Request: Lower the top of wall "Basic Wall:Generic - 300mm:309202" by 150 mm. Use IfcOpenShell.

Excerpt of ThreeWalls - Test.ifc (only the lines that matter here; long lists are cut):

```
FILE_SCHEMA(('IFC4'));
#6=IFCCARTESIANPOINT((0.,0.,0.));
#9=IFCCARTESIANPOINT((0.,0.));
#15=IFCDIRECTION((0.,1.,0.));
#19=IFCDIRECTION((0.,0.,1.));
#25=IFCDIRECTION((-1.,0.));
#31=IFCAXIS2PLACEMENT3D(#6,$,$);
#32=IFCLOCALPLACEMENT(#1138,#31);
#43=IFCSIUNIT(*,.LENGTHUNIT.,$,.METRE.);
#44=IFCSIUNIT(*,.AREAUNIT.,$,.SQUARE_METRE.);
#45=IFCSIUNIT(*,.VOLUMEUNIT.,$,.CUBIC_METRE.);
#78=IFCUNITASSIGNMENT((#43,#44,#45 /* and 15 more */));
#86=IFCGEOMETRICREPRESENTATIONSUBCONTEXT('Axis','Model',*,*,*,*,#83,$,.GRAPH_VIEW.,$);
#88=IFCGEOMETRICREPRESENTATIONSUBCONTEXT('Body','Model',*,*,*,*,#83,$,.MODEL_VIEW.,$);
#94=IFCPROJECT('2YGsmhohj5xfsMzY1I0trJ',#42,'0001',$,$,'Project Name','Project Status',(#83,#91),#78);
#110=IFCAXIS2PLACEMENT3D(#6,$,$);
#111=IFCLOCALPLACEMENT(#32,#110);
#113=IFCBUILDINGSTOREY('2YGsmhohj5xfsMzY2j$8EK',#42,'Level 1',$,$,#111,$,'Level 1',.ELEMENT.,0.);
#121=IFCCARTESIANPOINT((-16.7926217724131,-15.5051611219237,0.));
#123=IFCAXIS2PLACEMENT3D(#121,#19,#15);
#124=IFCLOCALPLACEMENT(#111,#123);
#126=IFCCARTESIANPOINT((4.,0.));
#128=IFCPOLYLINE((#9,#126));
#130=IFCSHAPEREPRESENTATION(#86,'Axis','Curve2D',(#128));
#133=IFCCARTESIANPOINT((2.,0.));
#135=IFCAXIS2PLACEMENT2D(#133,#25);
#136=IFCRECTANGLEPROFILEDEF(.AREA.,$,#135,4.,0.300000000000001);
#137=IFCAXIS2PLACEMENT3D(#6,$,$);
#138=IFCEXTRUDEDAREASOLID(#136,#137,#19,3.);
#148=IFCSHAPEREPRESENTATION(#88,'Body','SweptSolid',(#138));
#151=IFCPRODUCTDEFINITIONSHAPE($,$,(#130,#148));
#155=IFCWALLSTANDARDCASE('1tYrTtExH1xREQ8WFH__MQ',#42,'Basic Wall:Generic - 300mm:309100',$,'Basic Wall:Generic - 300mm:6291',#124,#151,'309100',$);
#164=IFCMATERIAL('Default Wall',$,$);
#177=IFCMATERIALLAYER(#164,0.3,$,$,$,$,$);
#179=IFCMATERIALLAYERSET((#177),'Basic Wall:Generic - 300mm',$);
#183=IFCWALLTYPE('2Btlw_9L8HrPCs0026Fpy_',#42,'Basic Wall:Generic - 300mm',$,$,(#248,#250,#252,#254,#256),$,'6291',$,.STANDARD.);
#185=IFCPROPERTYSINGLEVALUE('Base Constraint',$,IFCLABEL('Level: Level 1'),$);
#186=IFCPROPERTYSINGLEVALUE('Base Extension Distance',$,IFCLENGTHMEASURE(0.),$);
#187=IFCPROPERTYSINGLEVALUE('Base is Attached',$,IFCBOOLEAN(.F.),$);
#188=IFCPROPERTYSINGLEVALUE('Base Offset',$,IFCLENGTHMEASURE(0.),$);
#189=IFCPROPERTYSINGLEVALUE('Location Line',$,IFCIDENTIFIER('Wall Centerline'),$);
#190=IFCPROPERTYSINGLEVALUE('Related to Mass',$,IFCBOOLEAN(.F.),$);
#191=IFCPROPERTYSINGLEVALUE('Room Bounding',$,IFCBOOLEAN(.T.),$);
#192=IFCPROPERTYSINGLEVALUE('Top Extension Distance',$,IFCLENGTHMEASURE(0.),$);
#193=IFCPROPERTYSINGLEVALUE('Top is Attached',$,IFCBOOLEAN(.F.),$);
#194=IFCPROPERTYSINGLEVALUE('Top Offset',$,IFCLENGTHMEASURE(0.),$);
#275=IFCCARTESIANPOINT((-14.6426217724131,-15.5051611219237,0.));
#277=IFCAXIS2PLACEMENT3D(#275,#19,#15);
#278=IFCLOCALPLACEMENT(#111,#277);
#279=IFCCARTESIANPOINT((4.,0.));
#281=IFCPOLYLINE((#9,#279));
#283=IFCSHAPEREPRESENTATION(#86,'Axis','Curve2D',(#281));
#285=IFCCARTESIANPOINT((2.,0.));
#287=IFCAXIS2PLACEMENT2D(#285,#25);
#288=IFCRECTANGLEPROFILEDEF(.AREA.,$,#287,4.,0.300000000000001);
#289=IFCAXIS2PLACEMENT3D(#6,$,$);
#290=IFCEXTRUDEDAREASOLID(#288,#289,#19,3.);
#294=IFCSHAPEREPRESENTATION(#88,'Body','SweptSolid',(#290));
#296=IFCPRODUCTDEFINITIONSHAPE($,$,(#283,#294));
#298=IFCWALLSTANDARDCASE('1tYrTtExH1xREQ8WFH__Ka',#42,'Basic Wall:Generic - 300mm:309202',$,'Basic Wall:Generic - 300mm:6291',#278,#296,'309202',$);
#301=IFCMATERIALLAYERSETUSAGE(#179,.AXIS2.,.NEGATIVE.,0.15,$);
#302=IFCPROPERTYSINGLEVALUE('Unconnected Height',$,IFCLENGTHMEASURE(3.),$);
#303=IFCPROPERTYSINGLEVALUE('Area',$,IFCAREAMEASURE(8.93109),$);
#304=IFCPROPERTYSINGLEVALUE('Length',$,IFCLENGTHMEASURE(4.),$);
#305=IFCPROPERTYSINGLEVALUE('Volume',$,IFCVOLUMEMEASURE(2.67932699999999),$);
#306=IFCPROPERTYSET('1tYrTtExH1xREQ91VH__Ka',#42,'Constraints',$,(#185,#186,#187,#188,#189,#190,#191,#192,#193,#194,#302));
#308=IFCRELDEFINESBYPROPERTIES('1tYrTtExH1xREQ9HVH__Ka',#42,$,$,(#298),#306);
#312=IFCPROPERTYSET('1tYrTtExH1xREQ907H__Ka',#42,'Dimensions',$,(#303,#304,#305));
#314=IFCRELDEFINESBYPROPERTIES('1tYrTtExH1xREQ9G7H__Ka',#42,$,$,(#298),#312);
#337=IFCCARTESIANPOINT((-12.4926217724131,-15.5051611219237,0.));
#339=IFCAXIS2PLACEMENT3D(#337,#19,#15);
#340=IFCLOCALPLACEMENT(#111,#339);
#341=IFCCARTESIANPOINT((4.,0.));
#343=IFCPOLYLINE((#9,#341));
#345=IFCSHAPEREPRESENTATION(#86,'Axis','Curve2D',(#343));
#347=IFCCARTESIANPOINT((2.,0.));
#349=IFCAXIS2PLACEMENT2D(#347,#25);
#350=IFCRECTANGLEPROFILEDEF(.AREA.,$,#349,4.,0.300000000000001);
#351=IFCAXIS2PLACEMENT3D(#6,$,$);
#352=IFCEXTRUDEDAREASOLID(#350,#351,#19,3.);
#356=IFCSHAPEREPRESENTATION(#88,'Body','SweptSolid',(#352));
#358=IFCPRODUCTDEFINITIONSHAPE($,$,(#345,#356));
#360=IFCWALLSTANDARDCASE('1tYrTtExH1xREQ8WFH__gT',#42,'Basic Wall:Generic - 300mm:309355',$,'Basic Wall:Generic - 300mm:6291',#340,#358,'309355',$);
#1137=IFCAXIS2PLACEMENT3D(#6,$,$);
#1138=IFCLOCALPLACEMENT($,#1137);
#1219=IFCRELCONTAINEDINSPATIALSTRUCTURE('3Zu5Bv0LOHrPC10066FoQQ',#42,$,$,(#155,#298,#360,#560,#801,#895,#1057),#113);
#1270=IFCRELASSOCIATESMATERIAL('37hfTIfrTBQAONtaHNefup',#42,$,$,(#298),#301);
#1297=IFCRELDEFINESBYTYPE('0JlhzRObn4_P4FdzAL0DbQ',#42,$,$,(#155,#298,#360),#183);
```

```python
import ifcopenshell
import ifcopenshell.api.pset
import ifcopenshell.geom
import ifcopenshell.util.element
import ifcopenshell.util.representation
import ifcopenshell.util.shape
import ifcopenshell.util.unit

model = ifcopenshell.open("ThreeWalls - Test.ifc")
area_scale = ifcopenshell.util.unit.calculate_unit_scale(model, "AREAUNIT")
volume_scale = ifcopenshell.util.unit.calculate_unit_scale(model, "VOLUMEUNIT")
settings = ifcopenshell.geom.settings()


def volume(element):
    """Net volume in cubic metres, openings subtracted."""
    shape = ifcopenshell.geom.create_shape(settings, element)
    return ifcopenshell.util.shape.get_volume(shape.geometry)


wall = model.by_id(298)
before = volume(wall)

body = ifcopenshell.util.representation.get_representation(wall, "Model", "Body")
solid = body.Items[0]
old_height = solid.Depth
solid.Depth -= 0.15
after = volume(wall)
thickness = 0.3  # wall thickness in metres

# Update the stored height, areas and volumes.
pset = model.by_id(ifcopenshell.util.element.get_pset(wall, "Constraints", should_inherit=False)["id"])
ifcopenshell.api.pset.edit_pset(model, pset=pset, properties={
    "Unconnected Height": model.create_entity("IfcLengthMeasure", solid.Depth),
})
pset = model.by_id(ifcopenshell.util.element.get_pset(wall, "Dimensions", should_inherit=False)["id"])
ifcopenshell.api.pset.edit_pset(model, pset=pset, properties={
    "Area": model.create_entity("IfcAreaMeasure", after / thickness / area_scale),
    "Volume": model.create_entity("IfcVolumeMeasure", after / volume_scale),
})

print(f"height {old_height:g} -> {solid.Depth:g}, volume {before:.3f} -> {after:.3f} m3")

model.write("ThreeWalls - Test_rev.ifc")
```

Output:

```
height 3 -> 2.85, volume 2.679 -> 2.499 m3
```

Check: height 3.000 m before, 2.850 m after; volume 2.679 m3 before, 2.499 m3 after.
